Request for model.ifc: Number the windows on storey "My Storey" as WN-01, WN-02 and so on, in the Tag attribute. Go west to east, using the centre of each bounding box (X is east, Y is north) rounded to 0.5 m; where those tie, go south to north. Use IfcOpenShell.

First a look at what the model holds.

```python
import ifcopenshell
import ifcopenshell.util.element
import ifcopenshell.util.placement

model = ifcopenshell.open("model.ifc")
print(model.schema)
storey = next(s for s in model.by_type("IfcBuildingStorey") if s.Name == "My Storey")
windows = [e for e in ifcopenshell.util.element.get_decomposition(storey) if e.is_a("IfcWindow")]
for e in sorted(windows, key=lambda e: e.id()):
    origin = ifcopenshell.util.placement.get_local_placement(e.ObjectPlacement)[:3, 3]
    print(e.id(), e.Tag, e.Name, origin.round(2) + 0.0, sep=" | ")
```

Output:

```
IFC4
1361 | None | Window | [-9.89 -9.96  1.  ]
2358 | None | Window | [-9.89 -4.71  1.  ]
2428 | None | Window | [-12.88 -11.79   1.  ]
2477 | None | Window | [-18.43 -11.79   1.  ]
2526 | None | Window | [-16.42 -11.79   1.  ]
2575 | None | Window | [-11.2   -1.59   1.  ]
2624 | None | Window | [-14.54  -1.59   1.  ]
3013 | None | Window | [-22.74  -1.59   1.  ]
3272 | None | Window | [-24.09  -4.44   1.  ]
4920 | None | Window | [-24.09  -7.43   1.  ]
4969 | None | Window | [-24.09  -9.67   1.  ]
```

```python
import ifcopenshell
import ifcopenshell.geom
import ifcopenshell.util.element
import ifcopenshell.util.shape

model = ifcopenshell.open("model.ifc")
settings = ifcopenshell.geom.settings()
settings.set("use-world-coords", True)


def centre(element):
    shape = ifcopenshell.geom.create_shape(settings, element)
    return ifcopenshell.util.shape.get_bbox_centroid(shape.geometry)


storey = next(s for s in model.by_type("IfcBuildingStorey") if s.Name == "My Storey")
windows = [e for e in ifcopenshell.util.element.get_decomposition(storey) if e.is_a("IfcWindow")]

# Insertion points can sit at a corner or the storey origin, so sort by the geometry (in metres).
centres = {e: centre(e) for e in windows}
windows.sort(key=lambda e: (round(centres[e][0] / 0.5), centres[e][1]))

for i, e in enumerate(windows, start=1):
    number = f"WN-{i:02d}"
    e.Tag = number
    print(e.id(), number)

model.write("model-out.ifc")
```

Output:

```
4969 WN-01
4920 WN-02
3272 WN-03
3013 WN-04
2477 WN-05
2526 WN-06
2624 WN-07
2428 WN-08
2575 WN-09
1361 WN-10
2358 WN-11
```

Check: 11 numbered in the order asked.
